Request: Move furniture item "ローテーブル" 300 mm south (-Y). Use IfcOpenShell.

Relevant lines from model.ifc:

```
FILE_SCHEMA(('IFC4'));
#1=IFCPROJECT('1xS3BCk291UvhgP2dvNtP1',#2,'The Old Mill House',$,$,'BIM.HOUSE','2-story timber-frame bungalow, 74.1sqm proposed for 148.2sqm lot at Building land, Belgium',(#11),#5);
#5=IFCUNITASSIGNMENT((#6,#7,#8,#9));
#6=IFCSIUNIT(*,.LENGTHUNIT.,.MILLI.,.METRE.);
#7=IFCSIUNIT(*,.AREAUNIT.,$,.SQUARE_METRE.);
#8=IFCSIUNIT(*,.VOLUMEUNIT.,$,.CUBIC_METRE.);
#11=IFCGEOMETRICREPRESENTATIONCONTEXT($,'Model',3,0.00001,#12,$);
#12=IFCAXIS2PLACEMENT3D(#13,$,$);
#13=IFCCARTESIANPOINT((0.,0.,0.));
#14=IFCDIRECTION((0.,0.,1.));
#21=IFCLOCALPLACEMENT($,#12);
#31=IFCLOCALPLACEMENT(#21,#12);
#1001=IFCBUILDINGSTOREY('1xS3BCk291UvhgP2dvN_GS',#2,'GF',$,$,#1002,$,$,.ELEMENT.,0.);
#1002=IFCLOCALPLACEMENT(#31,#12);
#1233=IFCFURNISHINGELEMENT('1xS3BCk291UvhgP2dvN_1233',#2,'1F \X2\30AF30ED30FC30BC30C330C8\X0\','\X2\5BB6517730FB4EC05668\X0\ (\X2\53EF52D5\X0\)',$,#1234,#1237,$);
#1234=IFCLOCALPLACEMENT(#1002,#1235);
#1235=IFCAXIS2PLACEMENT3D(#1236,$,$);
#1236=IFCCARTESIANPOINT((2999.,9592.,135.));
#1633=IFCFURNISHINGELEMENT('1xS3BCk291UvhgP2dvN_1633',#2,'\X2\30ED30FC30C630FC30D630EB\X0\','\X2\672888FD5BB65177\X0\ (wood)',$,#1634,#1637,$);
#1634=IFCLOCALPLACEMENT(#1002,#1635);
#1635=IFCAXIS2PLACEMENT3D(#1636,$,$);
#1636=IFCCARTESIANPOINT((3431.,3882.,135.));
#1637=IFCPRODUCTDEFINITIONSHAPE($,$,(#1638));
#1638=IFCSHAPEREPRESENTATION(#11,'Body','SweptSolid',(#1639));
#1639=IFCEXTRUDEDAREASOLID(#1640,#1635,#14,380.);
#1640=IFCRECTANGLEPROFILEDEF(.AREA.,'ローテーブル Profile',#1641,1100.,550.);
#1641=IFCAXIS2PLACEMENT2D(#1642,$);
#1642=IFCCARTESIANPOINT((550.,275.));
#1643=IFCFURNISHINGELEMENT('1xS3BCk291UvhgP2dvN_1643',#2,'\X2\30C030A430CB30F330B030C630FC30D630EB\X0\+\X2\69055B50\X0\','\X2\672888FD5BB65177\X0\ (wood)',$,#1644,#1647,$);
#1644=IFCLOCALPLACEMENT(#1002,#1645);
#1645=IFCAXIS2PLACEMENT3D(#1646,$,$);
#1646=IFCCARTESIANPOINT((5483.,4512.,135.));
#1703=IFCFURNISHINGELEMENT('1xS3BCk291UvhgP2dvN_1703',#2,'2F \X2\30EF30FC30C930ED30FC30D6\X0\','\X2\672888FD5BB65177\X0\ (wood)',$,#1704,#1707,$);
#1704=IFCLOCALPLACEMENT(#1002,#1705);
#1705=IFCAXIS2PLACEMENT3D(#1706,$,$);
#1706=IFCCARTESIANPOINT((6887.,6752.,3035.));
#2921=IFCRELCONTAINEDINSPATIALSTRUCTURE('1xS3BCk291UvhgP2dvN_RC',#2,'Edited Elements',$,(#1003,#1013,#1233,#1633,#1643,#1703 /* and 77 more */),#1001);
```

```python
import ifcopenshell
import ifcopenshell.api.geometry
import ifcopenshell.util.placement
import ifcopenshell.util.unit

model = ifcopenshell.open("model.ifc")
unit_scale = ifcopenshell.util.unit.calculate_unit_scale(model)

item = model.by_guid("1xS3BCk291UvhgP2dvN_1633")
matrix = ifcopenshell.util.placement.get_local_placement(item.ObjectPlacement)
matrix[1, 3] -= 0.3 / unit_scale
ifcopenshell.api.geometry.edit_object_placement(model, product=item, matrix=matrix, is_si=False)

print(ifcopenshell.util.placement.get_local_placement(item.ObjectPlacement).round(3) + 0.0)

model.write("model-out.ifc")
```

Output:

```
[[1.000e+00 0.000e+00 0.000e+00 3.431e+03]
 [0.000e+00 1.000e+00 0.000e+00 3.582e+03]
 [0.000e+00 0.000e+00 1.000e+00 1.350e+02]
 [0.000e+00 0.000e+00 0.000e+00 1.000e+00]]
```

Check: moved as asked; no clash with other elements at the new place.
